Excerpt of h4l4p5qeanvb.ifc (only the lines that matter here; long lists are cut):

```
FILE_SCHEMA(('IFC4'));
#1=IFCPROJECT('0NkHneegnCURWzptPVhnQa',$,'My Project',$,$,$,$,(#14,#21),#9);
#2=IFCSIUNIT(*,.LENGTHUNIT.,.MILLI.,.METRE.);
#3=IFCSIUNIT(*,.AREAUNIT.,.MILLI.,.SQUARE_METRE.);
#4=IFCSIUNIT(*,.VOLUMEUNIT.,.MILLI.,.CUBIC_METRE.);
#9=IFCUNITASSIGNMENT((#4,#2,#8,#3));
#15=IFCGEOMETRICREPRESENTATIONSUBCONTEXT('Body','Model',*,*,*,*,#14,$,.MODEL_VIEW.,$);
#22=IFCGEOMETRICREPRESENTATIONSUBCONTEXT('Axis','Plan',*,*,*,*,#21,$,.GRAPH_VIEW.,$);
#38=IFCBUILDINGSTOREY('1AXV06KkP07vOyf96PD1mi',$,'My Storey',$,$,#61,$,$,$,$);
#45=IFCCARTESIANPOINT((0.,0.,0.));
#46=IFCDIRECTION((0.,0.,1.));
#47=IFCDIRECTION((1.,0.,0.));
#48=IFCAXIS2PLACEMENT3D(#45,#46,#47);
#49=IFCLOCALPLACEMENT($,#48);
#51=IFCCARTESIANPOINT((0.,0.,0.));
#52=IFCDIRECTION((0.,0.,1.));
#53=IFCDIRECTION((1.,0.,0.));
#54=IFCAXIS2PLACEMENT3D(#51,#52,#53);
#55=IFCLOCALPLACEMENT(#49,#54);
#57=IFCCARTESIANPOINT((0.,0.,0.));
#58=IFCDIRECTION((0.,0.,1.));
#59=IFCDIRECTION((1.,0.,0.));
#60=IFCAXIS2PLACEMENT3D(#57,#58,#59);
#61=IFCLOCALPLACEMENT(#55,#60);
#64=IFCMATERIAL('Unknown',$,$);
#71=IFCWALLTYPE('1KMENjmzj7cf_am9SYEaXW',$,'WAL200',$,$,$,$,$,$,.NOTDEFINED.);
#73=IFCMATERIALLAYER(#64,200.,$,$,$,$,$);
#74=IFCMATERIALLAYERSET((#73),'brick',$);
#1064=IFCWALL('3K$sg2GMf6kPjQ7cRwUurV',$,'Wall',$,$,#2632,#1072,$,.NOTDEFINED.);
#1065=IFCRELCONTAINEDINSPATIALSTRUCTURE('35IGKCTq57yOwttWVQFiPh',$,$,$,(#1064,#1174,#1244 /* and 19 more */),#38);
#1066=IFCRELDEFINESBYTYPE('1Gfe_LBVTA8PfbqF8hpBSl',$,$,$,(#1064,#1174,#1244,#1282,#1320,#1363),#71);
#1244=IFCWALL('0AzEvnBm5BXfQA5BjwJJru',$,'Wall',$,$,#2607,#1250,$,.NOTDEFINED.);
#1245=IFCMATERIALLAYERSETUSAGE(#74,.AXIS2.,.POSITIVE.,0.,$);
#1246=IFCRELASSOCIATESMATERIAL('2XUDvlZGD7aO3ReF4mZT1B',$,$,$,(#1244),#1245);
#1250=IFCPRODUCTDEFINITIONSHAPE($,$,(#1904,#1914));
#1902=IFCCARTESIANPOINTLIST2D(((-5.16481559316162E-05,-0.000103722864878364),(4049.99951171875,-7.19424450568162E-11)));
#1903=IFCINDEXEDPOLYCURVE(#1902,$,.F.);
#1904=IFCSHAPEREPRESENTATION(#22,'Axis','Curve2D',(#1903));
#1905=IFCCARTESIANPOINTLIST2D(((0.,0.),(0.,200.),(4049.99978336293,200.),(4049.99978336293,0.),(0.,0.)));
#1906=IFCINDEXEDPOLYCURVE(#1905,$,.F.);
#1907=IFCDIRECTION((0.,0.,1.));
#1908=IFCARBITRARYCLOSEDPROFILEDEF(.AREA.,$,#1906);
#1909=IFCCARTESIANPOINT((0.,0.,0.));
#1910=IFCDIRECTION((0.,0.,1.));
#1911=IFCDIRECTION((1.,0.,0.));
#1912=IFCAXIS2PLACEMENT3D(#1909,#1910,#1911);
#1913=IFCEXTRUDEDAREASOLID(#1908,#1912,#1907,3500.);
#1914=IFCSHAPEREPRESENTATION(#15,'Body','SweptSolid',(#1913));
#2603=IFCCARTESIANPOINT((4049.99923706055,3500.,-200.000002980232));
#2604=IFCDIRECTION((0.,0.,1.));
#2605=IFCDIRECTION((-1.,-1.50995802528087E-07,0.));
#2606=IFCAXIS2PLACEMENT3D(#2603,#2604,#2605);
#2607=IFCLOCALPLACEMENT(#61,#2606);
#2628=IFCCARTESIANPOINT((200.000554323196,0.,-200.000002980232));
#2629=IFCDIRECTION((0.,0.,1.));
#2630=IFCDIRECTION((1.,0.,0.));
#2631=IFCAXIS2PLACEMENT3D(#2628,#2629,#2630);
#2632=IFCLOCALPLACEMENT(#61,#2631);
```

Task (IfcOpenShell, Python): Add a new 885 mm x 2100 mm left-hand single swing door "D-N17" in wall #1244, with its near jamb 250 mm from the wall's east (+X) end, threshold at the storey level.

```python
import numpy as np
import ifcopenshell
import ifcopenshell.api.feature
import ifcopenshell.api.geometry
import ifcopenshell.api.root
import ifcopenshell.api.spatial
import ifcopenshell.geom
import ifcopenshell.util.element
import ifcopenshell.util.placement
import ifcopenshell.util.representation
import ifcopenshell.util.shape
import ifcopenshell.util.unit

model = ifcopenshell.open("h4l4p5qeanvb.ifc")
unit_scale = ifcopenshell.util.unit.calculate_unit_scale(model)
settings = ifcopenshell.geom.settings()


def volume(element):
    """Net volume in cubic metres, openings subtracted."""
    shape = ifcopenshell.geom.create_shape(settings, element)
    return ifcopenshell.util.shape.get_volume(shape.geometry)


wall = model.by_guid("0AzEvnBm5BXfQA5BjwJJru")
storey = ifcopenshell.util.element.get_container(wall, ifc_class="IfcBuildingStorey")
context = ifcopenshell.util.representation.get_context(model, "Model", "Body", "MODEL_VIEW")
before = volume(wall)

width, height, from_end, sill = 0.885, 2.1, 0.25, 0.0  # metres

# The wall runs along its own X axis, and the end named is its -X end.
wall_shape = ifcopenshell.geom.create_shape(settings, wall)
x, y, z = ifcopenshell.util.shape.get_vertices(wall_shape.geometry).T
start = x.min() + from_end
face, thickness = float(y.min()), float(y.max() - y.min())
wall_matrix = ifcopenshell.util.placement.get_local_placement(wall.ObjectPlacement)
level = ifcopenshell.util.placement.get_local_placement(storey.ObjectPlacement)[2, 3]


def in_wall(x, y):
    """Placement at x, y metres in the wall's axes, at sill height."""
    matrix = wall_matrix.copy()
    matrix[:, 3] = wall_matrix @ np.array([x / unit_scale, y / unit_scale, 0.0, 1.0])
    matrix[2, 3] = level + sill / unit_scale
    return matrix


# Opening: a box that overshoots both wall faces by 50 mm.
opening = ifcopenshell.api.root.create_entity(model, ifc_class="IfcOpeningElement", predefined_type="OPENING")
box = ifcopenshell.api.geometry.add_wall_representation(
    model, context=context, length=width, height=height, thickness=thickness + 0.1
)
ifcopenshell.api.geometry.assign_representation(model, product=opening, representation=box)
ifcopenshell.api.geometry.edit_object_placement(model, product=opening, matrix=in_wall(start, face - 0.05), is_si=False)
ifcopenshell.api.feature.add_feature(model, feature=opening, element=wall)

door = ifcopenshell.api.root.create_entity(model, ifc_class="IfcDoor", name="D-N17", predefined_type="DOOR")
door.OverallWidth, door.OverallHeight = width / unit_scale, height / unit_scale
door.OperationType = "SINGLE_SWING_LEFT"
body = ifcopenshell.api.geometry.add_door_representation(
    model,
    context=context,
    overall_width=door.OverallWidth,
    overall_height=door.OverallHeight,
    operation_type="SINGLE_SWING_LEFT",
    lining_properties={"LiningDepth": thickness / unit_scale, "ThresholdDepth": thickness / unit_scale},
)
ifcopenshell.api.geometry.assign_representation(model, product=door, representation=body)
ifcopenshell.api.spatial.assign_container(model, products=[door], relating_structure=storey)
ifcopenshell.api.feature.add_filling(model, opening=opening, element=door)

# The lining spans the wall, so the door starts at the wall face.
ifcopenshell.api.geometry.edit_object_placement(model, product=door, matrix=in_wall(start, face), is_si=False)

after = volume(wall)

print(f"wall volume {before:.3f} -> {after:.3f} m3")

model.write("h4l4p5qeanvb_edited.ifc")
```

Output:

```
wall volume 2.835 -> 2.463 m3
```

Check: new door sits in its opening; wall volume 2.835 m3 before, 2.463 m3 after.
